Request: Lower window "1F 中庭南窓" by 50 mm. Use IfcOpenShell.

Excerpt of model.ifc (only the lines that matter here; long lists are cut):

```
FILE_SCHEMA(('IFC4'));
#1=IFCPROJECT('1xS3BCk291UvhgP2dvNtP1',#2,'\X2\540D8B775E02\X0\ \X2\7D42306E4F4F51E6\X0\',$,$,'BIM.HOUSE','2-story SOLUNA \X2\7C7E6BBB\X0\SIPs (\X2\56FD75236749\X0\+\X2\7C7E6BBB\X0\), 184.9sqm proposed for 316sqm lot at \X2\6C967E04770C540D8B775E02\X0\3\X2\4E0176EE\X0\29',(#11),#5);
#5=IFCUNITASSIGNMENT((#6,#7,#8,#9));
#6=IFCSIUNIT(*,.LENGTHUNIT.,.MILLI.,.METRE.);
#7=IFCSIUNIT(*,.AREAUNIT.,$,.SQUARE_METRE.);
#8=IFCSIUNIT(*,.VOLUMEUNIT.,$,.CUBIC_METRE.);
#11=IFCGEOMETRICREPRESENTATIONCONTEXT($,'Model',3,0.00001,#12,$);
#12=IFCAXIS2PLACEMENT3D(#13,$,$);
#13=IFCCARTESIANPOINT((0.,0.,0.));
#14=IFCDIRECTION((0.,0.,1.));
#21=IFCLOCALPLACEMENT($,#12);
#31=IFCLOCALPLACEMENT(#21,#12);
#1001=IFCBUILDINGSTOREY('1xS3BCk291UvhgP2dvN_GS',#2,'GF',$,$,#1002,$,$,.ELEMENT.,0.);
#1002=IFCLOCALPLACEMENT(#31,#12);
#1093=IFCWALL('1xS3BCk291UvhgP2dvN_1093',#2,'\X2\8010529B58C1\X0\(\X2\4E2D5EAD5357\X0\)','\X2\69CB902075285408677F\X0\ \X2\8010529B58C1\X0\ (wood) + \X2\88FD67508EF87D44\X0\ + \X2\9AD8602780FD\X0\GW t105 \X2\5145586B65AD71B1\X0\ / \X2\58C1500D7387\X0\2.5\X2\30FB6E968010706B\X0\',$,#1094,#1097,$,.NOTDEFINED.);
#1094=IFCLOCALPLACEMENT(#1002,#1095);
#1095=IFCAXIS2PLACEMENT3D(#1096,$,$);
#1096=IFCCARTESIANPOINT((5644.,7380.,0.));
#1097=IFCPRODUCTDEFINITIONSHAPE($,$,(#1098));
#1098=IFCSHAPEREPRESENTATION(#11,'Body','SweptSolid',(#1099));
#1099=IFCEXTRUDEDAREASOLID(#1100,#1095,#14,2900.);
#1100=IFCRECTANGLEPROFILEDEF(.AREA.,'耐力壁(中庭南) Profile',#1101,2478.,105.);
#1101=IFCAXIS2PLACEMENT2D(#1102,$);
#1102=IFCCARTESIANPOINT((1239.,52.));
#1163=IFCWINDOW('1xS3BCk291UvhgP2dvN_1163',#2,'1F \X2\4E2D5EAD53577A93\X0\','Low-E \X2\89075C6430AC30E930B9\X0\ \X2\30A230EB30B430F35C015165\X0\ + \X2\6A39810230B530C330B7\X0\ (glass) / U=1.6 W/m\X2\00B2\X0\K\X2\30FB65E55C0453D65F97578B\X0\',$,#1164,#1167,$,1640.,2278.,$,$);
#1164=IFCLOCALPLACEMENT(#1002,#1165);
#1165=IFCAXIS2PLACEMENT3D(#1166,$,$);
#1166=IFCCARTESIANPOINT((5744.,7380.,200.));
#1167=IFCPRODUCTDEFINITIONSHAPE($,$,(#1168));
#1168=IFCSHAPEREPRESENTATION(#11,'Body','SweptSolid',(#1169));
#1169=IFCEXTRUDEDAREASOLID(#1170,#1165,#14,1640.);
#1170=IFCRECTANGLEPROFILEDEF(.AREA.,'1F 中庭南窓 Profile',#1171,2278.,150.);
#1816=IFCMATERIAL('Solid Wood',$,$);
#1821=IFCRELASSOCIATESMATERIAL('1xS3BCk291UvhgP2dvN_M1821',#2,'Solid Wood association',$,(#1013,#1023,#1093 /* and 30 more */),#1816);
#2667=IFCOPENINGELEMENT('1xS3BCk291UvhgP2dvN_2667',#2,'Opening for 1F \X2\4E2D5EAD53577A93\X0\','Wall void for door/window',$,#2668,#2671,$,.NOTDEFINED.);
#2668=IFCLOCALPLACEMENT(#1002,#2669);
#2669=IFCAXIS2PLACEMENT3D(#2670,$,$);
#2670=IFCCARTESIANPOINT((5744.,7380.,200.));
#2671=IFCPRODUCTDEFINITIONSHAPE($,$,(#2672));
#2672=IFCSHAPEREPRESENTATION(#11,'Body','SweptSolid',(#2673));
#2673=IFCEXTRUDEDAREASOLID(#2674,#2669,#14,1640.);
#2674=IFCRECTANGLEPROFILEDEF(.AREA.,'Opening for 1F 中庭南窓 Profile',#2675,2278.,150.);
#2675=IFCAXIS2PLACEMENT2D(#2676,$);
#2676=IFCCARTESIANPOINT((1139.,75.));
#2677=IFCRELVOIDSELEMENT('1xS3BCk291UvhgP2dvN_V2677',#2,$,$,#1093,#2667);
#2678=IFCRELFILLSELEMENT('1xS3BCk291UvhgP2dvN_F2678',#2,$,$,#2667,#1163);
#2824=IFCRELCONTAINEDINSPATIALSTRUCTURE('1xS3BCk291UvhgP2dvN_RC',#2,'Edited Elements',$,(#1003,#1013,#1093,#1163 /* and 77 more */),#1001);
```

```python
import numpy as np
import ifcopenshell
import ifcopenshell.api.geometry
import ifcopenshell.util.placement
import ifcopenshell.util.unit

model = ifcopenshell.open("model.ifc")
unit_scale = ifcopenshell.util.unit.calculate_unit_scale(model)

window = model.by_guid("1xS3BCk291UvhgP2dvN_1163")
opening = window.FillsVoids[0].RelatingOpeningElement
dz = -0.05 / unit_scale

shift = np.array([0.0, 0.0, dz])
# The window is not placed relative to its opening, so move both.
for product in (opening, window):
    matrix = ifcopenshell.util.placement.get_local_placement(product.ObjectPlacement)
    matrix[:3, 3] += shift
    ifcopenshell.api.geometry.edit_object_placement(model, product=product, matrix=matrix, is_si=False)

print(f"moved by {dz * unit_scale:+.3f} m")

model.write("model_v2.ifc")
```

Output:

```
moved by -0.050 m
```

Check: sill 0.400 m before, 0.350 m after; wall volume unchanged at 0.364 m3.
